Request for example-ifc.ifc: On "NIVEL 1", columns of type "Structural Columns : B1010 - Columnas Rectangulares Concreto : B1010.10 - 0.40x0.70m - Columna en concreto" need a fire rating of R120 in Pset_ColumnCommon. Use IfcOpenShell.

First a look at what the model holds.

```python
import ifcopenshell
import ifcopenshell.util.element

model = ifcopenshell.open("example-ifc.ifc")
print(model.schema)
storey = next(s for s in model.by_type("IfcBuildingStorey") if s.Name == "NIVEL 1")
columns = [e for e in ifcopenshell.util.element.get_decomposition(storey) if e.is_a("IfcColumn")]
seen = {}
for e in columns:
    element_type = ifcopenshell.util.element.get_type(e)
    key = (element_type.Name if element_type != e and element_type else None, ifcopenshell.util.element.get_pset(e, "Pset_ColumnCommon", "FireRating"))
    seen[key] = seen.get(key, 0) + 1
for (name, value), count in sorted(seen.items(), key=str):
    print(count, "x", name, "|", value)
```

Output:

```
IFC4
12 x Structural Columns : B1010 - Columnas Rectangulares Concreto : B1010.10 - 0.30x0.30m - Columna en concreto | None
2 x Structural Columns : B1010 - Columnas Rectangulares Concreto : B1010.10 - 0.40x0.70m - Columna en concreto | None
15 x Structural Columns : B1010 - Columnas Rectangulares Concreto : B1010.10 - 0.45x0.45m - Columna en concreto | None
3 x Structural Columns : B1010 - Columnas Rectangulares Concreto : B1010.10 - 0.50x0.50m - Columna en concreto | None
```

```python
import ifcopenshell
import ifcopenshell.api.pset
import ifcopenshell.util.element

model = ifcopenshell.open("example-ifc.ifc")

storey = next(s for s in model.by_type("IfcBuildingStorey") if s.Name == "NIVEL 1")
columns = [e for e in ifcopenshell.util.element.get_decomposition(storey) if e.is_a("IfcColumn")]

count = 0
for e in columns:
    element_type = ifcopenshell.util.element.get_type(e)
    if element_type in (None, e) or element_type.Name != "Structural Columns : B1010 - Columnas Rectangulares Concreto : B1010.10 - 0.40x0.70m - Columna en concreto":
        continue
    # add_pset returns the element's existing set when there is one.
    pset = ifcopenshell.api.pset.add_pset(model, product=e, name="Pset_ColumnCommon")
    ifcopenshell.api.pset.edit_pset(model, pset=pset, properties={"FireRating": "R120"})
    count += 1

print(count, "columns updated")

model.write("example-ifc-out.ifc")
```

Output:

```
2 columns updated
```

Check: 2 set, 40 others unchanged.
